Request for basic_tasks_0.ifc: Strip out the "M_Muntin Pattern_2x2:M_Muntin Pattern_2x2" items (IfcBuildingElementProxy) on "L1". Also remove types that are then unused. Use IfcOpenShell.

First a look at what the model holds.

```python
import ifcopenshell
import ifcopenshell.util.element

model = ifcopenshell.open("basic_tasks_0.ifc")
print(model.schema)
storey = next(s for s in model.by_type("IfcBuildingStorey") if s.Name == "L1")
proxies = [e for e in ifcopenshell.util.element.get_decomposition(storey) if e.is_a("IfcBuildingElementProxy")]
seen = {}
for e in proxies:
    element_type = ifcopenshell.util.element.get_type(e)
    name = element_type.Name if element_type not in (None, e) else None
    seen[name] = seen.get(name, 0) + 1
for name, count in sorted(seen.items(), key=str):
    print(count, "x", name)
```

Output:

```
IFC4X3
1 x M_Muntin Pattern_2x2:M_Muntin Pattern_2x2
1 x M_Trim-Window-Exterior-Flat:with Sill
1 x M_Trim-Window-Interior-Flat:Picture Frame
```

```python
import ifcopenshell
import ifcopenshell.api.root
import ifcopenshell.util.element

model = ifcopenshell.open("basic_tasks_0.ifc")

storey = next(s for s in model.by_type("IfcBuildingStorey") if s.Name == "L1")
proxies = [e for e in ifcopenshell.util.element.get_decomposition(storey) if e.is_a("IfcBuildingElementProxy")]
targets = [e for e in proxies if (t := ifcopenshell.util.element.get_type(e)) not in (None, e) and t.Name == "M_Muntin Pattern_2x2:M_Muntin Pattern_2x2"]
types = {ifcopenshell.util.element.get_type(e) for e in targets} - {None, *targets}

for e in targets:
    ifcopenshell.api.root.remove_product(model, product=e)
print(len(targets), "removed")

unused = [t for t in types if not ifcopenshell.util.element.get_types(t)]
for t in unused:
    ifcopenshell.api.root.remove_product(model, product=t)
print(len(unused), "unused types removed")

model.write("basic_tasks_0_rev.ifc")
```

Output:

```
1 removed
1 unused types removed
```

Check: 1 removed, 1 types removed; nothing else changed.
